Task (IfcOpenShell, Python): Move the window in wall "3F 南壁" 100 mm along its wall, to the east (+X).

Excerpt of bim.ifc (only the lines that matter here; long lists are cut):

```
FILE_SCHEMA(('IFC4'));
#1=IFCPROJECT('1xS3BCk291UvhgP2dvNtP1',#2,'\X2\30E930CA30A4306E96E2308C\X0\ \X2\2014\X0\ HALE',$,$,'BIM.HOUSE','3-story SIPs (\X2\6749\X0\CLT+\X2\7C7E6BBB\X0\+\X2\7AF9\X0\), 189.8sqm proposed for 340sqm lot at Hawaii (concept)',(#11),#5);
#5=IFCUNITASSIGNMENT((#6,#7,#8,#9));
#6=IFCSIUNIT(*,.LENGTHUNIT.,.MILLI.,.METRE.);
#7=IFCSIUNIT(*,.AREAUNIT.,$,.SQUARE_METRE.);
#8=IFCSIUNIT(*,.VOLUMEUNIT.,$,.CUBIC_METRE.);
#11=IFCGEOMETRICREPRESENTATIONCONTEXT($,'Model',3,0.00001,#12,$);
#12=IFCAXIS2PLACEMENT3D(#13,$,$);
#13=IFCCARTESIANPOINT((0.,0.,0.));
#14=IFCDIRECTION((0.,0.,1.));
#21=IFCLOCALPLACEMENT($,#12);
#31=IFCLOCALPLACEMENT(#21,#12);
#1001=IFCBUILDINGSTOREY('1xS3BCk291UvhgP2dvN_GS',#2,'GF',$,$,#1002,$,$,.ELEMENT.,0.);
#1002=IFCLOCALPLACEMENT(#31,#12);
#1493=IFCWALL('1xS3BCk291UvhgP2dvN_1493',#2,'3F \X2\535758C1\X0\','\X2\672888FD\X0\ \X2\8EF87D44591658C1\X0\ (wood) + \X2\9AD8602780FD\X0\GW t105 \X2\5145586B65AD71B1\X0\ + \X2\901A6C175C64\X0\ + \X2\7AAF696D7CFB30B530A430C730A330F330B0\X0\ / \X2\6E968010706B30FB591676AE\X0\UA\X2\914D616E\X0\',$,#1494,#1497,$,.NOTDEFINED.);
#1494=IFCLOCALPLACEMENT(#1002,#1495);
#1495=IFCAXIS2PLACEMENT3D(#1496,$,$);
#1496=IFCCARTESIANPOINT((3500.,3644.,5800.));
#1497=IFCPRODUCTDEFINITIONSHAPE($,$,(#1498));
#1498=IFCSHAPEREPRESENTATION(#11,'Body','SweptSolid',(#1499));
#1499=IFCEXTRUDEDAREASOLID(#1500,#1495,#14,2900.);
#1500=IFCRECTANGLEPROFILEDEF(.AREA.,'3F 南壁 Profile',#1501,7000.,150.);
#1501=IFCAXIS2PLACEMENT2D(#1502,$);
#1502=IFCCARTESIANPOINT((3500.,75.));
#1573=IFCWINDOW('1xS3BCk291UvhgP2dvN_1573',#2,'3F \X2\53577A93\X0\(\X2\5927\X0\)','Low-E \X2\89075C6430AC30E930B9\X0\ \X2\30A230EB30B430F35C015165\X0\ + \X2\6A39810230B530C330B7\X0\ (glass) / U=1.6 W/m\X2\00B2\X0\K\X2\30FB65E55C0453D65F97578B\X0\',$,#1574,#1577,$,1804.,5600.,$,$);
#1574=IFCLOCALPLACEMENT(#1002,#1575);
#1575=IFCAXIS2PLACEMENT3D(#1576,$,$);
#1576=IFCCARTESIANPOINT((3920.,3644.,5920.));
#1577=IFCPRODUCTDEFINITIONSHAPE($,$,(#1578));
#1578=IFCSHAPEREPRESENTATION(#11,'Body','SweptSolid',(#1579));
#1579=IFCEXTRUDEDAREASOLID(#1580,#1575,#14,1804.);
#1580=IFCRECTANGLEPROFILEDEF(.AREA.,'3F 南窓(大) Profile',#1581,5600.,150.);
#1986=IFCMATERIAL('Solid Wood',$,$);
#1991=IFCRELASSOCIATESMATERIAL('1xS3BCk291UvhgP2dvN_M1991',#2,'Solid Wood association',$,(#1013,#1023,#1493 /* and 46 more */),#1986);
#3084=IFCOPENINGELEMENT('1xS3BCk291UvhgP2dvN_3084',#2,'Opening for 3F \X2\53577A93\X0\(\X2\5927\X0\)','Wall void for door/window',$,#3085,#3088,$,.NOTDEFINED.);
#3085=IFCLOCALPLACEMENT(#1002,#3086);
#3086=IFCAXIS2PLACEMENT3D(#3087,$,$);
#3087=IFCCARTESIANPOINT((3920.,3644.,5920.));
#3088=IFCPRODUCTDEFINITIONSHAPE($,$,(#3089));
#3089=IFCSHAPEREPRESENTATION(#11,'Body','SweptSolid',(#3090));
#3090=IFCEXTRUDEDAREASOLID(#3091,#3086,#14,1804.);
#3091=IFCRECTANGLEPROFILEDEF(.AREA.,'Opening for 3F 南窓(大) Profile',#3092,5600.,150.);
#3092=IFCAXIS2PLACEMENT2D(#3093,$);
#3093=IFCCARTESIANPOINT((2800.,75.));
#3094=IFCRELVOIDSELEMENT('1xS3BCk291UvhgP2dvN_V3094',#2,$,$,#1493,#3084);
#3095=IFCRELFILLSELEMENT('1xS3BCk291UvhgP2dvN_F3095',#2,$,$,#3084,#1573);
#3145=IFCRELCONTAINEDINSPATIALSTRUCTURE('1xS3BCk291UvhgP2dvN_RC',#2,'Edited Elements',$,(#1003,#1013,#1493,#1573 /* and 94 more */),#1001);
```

```python
import ifcopenshell
import ifcopenshell.api.geometry
import ifcopenshell.util.placement
import ifcopenshell.util.unit

model = ifcopenshell.open("bim.ifc")
unit_scale = ifcopenshell.util.unit.calculate_unit_scale(model)

window = model.by_guid("1xS3BCk291UvhgP2dvN_1573")
opening = window.FillsVoids[0].RelatingOpeningElement
wall = opening.VoidsElements[0].RelatingBuildingElement

wall_matrix = ifcopenshell.util.placement.get_local_placement(wall.ObjectPlacement)
shift = wall_matrix[:3, 0] * 0.1 / unit_scale
before = ifcopenshell.util.placement.get_local_placement(window.ObjectPlacement)[:3, 3].copy()

# The window is not placed relative to its opening, so move both.
for product in (opening, window):
    matrix = ifcopenshell.util.placement.get_local_placement(product.ObjectPlacement)
    matrix[:3, 3] += shift
    ifcopenshell.api.geometry.edit_object_placement(model, product=product, matrix=matrix, is_si=False)

after = ifcopenshell.util.placement.get_local_placement(window.ObjectPlacement)[:3, 3]
print("window moved by", (after - before).round(3) + 0.0)

model.write("bim_edited.ifc")
```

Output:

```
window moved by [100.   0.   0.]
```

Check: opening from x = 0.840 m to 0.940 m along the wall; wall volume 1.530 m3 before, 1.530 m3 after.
